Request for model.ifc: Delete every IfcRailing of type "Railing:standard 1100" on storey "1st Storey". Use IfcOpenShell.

First a look at what the model holds.

```python
import ifcopenshell
import ifcopenshell.util.element

model = ifcopenshell.open("model.ifc")
print(model.schema)
storey = next(s for s in model.by_type("IfcBuildingStorey") if s.Name == "1st Storey")
railings = [e for e in ifcopenshell.util.element.get_decomposition(storey) if e.is_a("IfcRailing")]
seen = {}
for e in railings:
    element_type = ifcopenshell.util.element.get_type(e)
    name = element_type.Name if element_type not in (None, e) else None
    seen[name] = seen.get(name, 0) + 1
for name, count in sorted(seen.items(), key=str):
    print(count, "x", name)
```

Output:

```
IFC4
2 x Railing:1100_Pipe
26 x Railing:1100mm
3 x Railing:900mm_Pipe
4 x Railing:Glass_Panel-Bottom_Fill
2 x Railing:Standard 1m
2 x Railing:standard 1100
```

```python
import ifcopenshell
import ifcopenshell.api.root
import ifcopenshell.util.element

model = ifcopenshell.open("model.ifc")

storey = next(s for s in model.by_type("IfcBuildingStorey") if s.Name == "1st Storey")
railings = [e for e in ifcopenshell.util.element.get_decomposition(storey) if e.is_a("IfcRailing")]
targets = [e for e in railings if (t := ifcopenshell.util.element.get_type(e)) not in (None, e) and t.Name == "Railing:standard 1100"]

for e in targets:
    ifcopenshell.api.root.remove_product(model, product=e)
print(len(targets), "removed")

model.write("model_v2.ifc")
```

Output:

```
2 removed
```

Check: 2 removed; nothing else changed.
